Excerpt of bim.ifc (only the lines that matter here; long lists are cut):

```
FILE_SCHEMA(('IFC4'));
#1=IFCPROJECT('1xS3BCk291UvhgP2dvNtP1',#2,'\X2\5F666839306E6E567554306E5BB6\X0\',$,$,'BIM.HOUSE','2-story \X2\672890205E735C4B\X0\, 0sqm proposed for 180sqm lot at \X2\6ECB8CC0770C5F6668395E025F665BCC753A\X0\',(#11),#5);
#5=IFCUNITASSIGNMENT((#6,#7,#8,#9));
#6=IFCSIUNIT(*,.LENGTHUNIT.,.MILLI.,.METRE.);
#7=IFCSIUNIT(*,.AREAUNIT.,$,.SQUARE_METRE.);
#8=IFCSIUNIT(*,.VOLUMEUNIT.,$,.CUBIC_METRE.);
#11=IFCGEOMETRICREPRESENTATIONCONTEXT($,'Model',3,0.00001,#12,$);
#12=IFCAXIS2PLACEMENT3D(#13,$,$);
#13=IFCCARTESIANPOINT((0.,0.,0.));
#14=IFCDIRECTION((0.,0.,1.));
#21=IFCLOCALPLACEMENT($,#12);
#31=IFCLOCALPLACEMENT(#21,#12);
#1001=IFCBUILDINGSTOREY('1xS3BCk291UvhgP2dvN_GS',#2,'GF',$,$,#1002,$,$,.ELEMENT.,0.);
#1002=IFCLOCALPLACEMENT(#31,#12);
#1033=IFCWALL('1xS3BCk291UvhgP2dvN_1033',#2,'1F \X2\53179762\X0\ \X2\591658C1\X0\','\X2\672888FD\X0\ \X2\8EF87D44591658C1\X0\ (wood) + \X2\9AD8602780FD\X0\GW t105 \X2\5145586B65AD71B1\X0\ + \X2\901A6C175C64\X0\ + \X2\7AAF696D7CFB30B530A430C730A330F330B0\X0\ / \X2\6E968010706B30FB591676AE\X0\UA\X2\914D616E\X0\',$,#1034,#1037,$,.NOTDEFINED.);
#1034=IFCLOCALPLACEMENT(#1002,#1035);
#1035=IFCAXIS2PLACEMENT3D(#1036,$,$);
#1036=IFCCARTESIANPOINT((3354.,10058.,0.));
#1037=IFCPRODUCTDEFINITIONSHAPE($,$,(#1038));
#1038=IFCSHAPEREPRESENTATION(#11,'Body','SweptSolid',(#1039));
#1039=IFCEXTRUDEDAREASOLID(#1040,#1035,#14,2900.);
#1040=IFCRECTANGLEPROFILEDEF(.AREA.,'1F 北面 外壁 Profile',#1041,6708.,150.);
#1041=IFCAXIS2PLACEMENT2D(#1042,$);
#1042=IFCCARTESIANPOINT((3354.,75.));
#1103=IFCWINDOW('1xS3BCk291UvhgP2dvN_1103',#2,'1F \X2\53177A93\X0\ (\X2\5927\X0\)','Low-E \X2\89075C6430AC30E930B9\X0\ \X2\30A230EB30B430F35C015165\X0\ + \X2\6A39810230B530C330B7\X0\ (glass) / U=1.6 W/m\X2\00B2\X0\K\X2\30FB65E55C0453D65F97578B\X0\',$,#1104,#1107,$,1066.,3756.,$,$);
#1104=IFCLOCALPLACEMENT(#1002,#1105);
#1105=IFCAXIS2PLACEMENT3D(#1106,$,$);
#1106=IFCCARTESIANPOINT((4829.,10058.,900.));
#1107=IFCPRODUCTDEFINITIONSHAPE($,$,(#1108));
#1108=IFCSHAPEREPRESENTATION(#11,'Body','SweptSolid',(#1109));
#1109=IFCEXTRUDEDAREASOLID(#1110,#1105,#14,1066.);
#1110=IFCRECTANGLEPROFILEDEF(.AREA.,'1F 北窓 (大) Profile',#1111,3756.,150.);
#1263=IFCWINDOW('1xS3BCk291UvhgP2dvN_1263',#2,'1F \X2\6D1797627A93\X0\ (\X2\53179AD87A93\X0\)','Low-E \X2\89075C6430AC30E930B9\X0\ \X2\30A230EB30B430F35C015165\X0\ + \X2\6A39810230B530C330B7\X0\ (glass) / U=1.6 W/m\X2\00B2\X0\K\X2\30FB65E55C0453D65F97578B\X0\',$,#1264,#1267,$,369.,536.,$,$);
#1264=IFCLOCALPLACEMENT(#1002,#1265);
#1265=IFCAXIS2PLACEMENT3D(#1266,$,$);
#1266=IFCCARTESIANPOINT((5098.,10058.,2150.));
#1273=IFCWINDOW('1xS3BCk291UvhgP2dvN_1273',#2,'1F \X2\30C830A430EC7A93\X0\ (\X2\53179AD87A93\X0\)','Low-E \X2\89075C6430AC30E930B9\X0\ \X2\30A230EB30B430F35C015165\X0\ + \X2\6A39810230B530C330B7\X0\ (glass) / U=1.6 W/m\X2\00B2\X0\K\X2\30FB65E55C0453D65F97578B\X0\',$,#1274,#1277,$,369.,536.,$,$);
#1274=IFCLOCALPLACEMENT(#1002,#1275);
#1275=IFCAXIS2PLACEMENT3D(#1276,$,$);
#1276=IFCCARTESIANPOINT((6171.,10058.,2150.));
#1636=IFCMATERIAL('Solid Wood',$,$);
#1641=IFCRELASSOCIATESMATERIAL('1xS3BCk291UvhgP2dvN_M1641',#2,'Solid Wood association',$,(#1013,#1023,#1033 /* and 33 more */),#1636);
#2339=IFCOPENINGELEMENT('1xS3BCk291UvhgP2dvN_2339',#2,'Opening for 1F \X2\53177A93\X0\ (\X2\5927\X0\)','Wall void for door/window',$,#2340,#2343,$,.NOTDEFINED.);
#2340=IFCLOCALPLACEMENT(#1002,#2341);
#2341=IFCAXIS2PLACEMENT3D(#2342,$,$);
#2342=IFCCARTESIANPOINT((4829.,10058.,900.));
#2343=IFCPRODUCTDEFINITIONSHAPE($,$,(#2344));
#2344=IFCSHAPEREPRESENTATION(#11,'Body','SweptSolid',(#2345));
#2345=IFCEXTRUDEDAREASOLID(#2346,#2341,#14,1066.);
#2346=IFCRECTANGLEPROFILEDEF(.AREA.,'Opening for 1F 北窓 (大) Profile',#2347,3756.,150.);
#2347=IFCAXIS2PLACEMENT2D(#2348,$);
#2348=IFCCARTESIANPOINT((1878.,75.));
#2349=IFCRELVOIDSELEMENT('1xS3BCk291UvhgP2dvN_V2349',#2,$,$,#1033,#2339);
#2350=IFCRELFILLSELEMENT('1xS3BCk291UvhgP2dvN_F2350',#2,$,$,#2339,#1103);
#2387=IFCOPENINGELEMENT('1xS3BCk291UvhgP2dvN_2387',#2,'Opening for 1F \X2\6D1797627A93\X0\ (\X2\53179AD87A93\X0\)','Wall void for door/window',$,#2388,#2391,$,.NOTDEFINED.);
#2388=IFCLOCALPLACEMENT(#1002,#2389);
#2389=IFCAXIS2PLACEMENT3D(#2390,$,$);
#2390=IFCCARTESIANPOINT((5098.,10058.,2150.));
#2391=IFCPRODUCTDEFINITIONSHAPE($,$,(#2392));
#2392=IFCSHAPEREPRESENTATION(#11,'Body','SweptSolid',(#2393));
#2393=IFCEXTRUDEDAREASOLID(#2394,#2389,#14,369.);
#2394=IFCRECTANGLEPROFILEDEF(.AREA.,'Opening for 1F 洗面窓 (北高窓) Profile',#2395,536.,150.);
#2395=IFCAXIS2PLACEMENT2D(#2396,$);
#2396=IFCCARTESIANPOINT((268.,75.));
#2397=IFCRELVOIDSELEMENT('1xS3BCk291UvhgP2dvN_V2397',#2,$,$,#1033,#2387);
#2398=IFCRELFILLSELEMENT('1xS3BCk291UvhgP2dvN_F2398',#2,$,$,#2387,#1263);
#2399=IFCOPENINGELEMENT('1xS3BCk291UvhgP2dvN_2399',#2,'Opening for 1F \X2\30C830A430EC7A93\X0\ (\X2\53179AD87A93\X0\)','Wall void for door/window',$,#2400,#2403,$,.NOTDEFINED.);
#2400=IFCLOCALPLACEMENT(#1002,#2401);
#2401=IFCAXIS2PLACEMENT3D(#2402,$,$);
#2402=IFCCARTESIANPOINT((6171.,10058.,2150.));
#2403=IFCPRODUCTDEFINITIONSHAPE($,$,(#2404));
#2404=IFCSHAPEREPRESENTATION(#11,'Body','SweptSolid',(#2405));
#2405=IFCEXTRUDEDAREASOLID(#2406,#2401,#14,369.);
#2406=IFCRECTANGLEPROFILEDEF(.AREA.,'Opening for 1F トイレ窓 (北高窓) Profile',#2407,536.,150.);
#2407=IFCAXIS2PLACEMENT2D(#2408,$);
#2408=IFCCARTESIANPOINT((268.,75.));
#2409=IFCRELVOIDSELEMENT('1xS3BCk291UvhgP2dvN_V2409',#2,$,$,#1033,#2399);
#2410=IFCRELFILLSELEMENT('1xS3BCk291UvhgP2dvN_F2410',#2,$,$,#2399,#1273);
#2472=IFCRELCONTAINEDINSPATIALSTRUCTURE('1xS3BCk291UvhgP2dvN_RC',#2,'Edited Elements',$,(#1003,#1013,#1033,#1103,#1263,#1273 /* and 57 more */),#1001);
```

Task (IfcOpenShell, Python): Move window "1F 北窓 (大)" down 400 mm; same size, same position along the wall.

```python
import numpy as np
import ifcopenshell
import ifcopenshell.api.geometry
import ifcopenshell.util.placement
import ifcopenshell.util.unit

model = ifcopenshell.open("bim.ifc")
unit_scale = ifcopenshell.util.unit.calculate_unit_scale(model)

window = model.by_guid("1xS3BCk291UvhgP2dvN_1103")
opening = window.FillsVoids[0].RelatingOpeningElement
dz = -0.4 / unit_scale

shift = np.array([0.0, 0.0, dz])
# The window is not placed relative to its opening, so move both.
for product in (opening, window):
    matrix = ifcopenshell.util.placement.get_local_placement(product.ObjectPlacement)
    matrix[:3, 3] += shift
    ifcopenshell.api.geometry.edit_object_placement(model, product=product, matrix=matrix, is_si=False)

print(f"moved by {dz * unit_scale:+.3f} m")

model.write("bim_updated.ifc")
```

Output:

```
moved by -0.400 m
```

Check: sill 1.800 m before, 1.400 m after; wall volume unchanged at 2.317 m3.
